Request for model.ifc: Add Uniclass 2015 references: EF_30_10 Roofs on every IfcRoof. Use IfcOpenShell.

First a look at what the model holds.

```python
import ifcopenshell

model = ifcopenshell.open("model.ifc")
print(model.schema)
print("classifications:", [c.Name for c in model.by_type("IfcClassification")])
for ifc_class in ("IfcDoor", "IfcRoof", "IfcStair", "IfcWall", "IfcWindow"):
    print(ifc_class, len(model.by_type(ifc_class)))
```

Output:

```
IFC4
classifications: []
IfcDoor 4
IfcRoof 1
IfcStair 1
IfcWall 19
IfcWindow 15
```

```python
import ifcopenshell
import ifcopenshell.api.classification

model = ifcopenshell.open("model.ifc")

system = ifcopenshell.api.classification.add_classification(model, classification="Uniclass 2015")

codes = {
    "IfcRoof": ("EF_30_10", "Roofs"),
}
for ifc_class, (code, name) in codes.items():
    products = model.by_type(ifc_class)
    ifcopenshell.api.classification.add_reference(
        model, products=products, classification=system, identification=code, name=name
    )
    print(code, len(products))

model.write("model_rev.ifc")
```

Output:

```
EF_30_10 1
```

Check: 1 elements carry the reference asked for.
